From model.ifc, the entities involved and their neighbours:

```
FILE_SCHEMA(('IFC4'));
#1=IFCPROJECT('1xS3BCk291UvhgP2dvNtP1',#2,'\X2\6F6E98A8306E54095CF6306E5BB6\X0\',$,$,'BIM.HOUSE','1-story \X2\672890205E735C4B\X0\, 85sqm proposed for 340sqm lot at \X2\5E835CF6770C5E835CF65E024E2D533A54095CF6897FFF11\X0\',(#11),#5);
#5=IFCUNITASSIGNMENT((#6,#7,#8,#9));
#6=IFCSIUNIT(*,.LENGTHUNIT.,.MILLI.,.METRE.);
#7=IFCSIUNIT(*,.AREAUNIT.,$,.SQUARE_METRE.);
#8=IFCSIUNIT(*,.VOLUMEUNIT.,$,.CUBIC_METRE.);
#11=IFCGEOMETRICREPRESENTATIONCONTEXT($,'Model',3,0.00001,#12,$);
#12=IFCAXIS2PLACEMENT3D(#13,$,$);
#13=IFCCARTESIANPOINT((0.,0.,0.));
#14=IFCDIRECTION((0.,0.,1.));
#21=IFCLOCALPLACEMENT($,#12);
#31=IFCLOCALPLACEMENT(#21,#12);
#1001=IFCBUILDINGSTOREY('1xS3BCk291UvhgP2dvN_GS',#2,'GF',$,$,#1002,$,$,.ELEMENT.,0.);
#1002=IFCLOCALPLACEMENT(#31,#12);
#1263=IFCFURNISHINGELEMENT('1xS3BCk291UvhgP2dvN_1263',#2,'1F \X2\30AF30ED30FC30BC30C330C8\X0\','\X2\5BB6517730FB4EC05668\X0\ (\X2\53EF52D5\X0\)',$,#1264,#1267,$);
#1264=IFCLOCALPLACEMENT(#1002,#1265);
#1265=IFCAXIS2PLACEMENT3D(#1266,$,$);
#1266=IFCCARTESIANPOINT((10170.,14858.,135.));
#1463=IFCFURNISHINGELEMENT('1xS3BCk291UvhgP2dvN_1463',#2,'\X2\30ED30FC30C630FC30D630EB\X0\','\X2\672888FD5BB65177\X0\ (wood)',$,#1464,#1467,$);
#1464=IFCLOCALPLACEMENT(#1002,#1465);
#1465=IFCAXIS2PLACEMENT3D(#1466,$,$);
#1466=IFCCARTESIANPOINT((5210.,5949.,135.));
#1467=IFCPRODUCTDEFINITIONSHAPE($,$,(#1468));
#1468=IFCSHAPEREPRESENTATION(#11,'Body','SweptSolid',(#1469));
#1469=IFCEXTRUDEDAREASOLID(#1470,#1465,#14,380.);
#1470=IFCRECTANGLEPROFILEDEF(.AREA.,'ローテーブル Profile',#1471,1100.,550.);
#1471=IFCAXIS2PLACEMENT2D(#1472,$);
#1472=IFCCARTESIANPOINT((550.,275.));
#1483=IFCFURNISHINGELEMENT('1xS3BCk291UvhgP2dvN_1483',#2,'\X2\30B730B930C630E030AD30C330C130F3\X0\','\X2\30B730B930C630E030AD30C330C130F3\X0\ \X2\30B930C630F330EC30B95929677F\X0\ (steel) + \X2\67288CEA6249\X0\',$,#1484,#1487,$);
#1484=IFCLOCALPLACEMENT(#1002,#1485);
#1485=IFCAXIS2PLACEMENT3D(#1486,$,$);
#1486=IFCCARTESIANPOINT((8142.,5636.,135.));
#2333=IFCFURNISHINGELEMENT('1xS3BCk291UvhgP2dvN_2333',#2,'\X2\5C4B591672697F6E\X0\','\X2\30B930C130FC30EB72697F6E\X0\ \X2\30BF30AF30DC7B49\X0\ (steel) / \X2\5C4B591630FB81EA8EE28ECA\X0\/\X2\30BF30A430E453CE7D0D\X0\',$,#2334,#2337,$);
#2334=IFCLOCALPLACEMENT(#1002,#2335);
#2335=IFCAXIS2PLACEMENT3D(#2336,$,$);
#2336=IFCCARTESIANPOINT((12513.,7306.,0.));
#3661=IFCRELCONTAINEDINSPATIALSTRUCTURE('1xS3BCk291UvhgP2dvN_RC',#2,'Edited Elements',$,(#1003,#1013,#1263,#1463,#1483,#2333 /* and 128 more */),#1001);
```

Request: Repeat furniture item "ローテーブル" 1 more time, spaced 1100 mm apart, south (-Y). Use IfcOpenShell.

```python
import numpy as np
import ifcopenshell
import ifcopenshell.api.geometry
import ifcopenshell.api.root
import ifcopenshell.util.element
import ifcopenshell.util.placement
import ifcopenshell.util.unit

model = ifcopenshell.open("model.ifc")
unit_scale = ifcopenshell.util.unit.calculate_unit_scale(model)


def reuse_history(source, copy):
    """copy_class also copies each property set's owner history, people and application; keep the originals."""
    for rel in copy.IsDefinedBy:
        if rel.is_a("IfcRelDefinesByProperties") and (history := rel.RelatingPropertyDefinition.OwnerHistory):
            rel.RelatingPropertyDefinition.OwnerHistory = source.OwnerHistory
            ifcopenshell.util.element.remove_deep2(model, history)


source = model.by_guid("1xS3BCk291UvhgP2dvN_1463")
base = ifcopenshell.util.placement.get_local_placement(source.ObjectPlacement)
step = np.array([0.0, -1.0, 0.0]) * 1.1 / unit_scale

for i in range(1, 2):
    copy = ifcopenshell.api.root.copy_class(model, product=source)
    copy.Representation = ifcopenshell.util.element.copy_deep(
        model, source.Representation, exclude=["IfcGeometricRepresentationContext", "IfcRepresentationMap"]
    )
    reuse_history(source, copy)
    matrix = base.copy()
    matrix[:3, 3] += i * step
    print("added at", matrix[:3, 3].round(3) + 0.0)
    ifcopenshell.api.geometry.edit_object_placement(model, product=copy, matrix=matrix, is_si=False)

model.write("model_updated.ifc")
```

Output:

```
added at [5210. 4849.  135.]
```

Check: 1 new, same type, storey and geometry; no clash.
